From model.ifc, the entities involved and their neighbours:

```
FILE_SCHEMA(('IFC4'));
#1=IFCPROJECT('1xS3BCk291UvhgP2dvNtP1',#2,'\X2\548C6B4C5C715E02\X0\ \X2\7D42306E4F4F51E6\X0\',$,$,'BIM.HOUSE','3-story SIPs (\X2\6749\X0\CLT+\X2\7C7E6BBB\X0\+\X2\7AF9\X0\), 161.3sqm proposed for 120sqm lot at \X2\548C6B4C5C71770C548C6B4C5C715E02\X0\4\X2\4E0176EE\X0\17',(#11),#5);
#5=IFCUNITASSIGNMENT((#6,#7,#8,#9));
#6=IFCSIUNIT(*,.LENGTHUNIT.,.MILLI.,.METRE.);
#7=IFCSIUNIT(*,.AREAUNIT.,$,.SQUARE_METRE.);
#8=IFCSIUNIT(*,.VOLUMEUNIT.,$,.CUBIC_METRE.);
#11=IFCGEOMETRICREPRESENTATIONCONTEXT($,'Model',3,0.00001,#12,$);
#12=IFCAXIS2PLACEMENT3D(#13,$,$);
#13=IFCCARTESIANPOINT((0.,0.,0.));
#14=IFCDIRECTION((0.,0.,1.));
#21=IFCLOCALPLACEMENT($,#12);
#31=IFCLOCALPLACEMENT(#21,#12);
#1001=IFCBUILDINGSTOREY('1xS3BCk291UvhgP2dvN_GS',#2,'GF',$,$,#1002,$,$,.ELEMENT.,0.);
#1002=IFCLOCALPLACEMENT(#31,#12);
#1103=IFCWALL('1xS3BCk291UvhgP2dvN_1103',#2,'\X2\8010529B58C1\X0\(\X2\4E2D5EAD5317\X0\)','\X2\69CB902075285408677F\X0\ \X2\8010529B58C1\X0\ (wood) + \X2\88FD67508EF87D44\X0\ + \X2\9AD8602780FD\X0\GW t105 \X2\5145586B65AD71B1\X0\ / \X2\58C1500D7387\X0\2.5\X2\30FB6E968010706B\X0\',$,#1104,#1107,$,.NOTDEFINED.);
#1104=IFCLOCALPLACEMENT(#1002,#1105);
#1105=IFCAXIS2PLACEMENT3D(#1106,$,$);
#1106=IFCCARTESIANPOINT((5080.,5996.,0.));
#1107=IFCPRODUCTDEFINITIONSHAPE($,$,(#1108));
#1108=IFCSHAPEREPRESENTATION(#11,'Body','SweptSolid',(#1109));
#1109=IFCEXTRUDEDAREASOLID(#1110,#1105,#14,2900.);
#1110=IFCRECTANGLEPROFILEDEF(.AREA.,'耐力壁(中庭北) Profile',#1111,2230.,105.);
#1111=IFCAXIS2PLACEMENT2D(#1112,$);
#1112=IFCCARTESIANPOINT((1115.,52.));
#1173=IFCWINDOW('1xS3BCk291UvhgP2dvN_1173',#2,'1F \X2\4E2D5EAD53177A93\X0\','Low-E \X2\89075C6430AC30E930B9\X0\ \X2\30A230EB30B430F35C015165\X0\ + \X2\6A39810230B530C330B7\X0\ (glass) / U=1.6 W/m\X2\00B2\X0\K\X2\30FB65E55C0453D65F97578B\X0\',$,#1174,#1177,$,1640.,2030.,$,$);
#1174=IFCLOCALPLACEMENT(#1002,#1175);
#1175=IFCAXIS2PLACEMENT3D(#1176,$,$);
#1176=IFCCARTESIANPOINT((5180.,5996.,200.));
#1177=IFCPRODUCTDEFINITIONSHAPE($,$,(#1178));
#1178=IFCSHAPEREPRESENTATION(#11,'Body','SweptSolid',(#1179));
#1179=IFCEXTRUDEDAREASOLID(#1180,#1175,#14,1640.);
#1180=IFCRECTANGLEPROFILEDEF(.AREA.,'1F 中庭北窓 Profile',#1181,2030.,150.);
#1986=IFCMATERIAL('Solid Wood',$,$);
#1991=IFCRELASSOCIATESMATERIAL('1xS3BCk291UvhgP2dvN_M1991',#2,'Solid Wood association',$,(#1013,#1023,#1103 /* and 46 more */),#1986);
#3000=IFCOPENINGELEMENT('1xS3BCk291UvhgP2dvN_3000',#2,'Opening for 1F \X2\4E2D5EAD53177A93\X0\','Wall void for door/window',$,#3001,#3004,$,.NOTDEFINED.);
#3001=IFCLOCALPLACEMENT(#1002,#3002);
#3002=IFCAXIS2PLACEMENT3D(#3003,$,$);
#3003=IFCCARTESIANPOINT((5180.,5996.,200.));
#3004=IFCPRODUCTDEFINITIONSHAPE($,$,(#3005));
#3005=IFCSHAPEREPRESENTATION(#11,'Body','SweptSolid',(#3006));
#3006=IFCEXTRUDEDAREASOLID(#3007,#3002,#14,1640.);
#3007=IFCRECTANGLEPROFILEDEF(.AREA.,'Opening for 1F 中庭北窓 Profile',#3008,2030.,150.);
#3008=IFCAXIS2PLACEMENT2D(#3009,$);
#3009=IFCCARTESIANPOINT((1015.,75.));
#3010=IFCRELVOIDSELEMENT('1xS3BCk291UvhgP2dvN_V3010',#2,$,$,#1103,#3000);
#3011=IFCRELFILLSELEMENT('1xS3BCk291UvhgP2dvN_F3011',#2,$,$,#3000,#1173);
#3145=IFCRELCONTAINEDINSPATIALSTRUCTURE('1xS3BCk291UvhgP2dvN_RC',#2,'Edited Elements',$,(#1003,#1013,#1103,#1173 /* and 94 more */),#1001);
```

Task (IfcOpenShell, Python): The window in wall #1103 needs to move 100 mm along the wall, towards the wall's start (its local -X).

```python
import ifcopenshell
import ifcopenshell.api.geometry
import ifcopenshell.util.placement
import ifcopenshell.util.unit

model = ifcopenshell.open("model.ifc")
unit_scale = ifcopenshell.util.unit.calculate_unit_scale(model)

window = model.by_guid("1xS3BCk291UvhgP2dvN_1173")
opening = window.FillsVoids[0].RelatingOpeningElement
wall = opening.VoidsElements[0].RelatingBuildingElement

wall_matrix = ifcopenshell.util.placement.get_local_placement(wall.ObjectPlacement)
shift = wall_matrix[:3, 0] * -0.1 / unit_scale
before = ifcopenshell.util.placement.get_local_placement(window.ObjectPlacement)[:3, 3].copy()

# The window is not placed relative to its opening, so move both.
for product in (opening, window):
    matrix = ifcopenshell.util.placement.get_local_placement(product.ObjectPlacement)
    matrix[:3, 3] += shift
    ifcopenshell.api.geometry.edit_object_placement(model, product=product, matrix=matrix, is_si=False)

after = ifcopenshell.util.placement.get_local_placement(window.ObjectPlacement)[:3, 3]
print("window moved by", (after - before).round(3) + 0.0)

model.write("model_rev.ifc")
```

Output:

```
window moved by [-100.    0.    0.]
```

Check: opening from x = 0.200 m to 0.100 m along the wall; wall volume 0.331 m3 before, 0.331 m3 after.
